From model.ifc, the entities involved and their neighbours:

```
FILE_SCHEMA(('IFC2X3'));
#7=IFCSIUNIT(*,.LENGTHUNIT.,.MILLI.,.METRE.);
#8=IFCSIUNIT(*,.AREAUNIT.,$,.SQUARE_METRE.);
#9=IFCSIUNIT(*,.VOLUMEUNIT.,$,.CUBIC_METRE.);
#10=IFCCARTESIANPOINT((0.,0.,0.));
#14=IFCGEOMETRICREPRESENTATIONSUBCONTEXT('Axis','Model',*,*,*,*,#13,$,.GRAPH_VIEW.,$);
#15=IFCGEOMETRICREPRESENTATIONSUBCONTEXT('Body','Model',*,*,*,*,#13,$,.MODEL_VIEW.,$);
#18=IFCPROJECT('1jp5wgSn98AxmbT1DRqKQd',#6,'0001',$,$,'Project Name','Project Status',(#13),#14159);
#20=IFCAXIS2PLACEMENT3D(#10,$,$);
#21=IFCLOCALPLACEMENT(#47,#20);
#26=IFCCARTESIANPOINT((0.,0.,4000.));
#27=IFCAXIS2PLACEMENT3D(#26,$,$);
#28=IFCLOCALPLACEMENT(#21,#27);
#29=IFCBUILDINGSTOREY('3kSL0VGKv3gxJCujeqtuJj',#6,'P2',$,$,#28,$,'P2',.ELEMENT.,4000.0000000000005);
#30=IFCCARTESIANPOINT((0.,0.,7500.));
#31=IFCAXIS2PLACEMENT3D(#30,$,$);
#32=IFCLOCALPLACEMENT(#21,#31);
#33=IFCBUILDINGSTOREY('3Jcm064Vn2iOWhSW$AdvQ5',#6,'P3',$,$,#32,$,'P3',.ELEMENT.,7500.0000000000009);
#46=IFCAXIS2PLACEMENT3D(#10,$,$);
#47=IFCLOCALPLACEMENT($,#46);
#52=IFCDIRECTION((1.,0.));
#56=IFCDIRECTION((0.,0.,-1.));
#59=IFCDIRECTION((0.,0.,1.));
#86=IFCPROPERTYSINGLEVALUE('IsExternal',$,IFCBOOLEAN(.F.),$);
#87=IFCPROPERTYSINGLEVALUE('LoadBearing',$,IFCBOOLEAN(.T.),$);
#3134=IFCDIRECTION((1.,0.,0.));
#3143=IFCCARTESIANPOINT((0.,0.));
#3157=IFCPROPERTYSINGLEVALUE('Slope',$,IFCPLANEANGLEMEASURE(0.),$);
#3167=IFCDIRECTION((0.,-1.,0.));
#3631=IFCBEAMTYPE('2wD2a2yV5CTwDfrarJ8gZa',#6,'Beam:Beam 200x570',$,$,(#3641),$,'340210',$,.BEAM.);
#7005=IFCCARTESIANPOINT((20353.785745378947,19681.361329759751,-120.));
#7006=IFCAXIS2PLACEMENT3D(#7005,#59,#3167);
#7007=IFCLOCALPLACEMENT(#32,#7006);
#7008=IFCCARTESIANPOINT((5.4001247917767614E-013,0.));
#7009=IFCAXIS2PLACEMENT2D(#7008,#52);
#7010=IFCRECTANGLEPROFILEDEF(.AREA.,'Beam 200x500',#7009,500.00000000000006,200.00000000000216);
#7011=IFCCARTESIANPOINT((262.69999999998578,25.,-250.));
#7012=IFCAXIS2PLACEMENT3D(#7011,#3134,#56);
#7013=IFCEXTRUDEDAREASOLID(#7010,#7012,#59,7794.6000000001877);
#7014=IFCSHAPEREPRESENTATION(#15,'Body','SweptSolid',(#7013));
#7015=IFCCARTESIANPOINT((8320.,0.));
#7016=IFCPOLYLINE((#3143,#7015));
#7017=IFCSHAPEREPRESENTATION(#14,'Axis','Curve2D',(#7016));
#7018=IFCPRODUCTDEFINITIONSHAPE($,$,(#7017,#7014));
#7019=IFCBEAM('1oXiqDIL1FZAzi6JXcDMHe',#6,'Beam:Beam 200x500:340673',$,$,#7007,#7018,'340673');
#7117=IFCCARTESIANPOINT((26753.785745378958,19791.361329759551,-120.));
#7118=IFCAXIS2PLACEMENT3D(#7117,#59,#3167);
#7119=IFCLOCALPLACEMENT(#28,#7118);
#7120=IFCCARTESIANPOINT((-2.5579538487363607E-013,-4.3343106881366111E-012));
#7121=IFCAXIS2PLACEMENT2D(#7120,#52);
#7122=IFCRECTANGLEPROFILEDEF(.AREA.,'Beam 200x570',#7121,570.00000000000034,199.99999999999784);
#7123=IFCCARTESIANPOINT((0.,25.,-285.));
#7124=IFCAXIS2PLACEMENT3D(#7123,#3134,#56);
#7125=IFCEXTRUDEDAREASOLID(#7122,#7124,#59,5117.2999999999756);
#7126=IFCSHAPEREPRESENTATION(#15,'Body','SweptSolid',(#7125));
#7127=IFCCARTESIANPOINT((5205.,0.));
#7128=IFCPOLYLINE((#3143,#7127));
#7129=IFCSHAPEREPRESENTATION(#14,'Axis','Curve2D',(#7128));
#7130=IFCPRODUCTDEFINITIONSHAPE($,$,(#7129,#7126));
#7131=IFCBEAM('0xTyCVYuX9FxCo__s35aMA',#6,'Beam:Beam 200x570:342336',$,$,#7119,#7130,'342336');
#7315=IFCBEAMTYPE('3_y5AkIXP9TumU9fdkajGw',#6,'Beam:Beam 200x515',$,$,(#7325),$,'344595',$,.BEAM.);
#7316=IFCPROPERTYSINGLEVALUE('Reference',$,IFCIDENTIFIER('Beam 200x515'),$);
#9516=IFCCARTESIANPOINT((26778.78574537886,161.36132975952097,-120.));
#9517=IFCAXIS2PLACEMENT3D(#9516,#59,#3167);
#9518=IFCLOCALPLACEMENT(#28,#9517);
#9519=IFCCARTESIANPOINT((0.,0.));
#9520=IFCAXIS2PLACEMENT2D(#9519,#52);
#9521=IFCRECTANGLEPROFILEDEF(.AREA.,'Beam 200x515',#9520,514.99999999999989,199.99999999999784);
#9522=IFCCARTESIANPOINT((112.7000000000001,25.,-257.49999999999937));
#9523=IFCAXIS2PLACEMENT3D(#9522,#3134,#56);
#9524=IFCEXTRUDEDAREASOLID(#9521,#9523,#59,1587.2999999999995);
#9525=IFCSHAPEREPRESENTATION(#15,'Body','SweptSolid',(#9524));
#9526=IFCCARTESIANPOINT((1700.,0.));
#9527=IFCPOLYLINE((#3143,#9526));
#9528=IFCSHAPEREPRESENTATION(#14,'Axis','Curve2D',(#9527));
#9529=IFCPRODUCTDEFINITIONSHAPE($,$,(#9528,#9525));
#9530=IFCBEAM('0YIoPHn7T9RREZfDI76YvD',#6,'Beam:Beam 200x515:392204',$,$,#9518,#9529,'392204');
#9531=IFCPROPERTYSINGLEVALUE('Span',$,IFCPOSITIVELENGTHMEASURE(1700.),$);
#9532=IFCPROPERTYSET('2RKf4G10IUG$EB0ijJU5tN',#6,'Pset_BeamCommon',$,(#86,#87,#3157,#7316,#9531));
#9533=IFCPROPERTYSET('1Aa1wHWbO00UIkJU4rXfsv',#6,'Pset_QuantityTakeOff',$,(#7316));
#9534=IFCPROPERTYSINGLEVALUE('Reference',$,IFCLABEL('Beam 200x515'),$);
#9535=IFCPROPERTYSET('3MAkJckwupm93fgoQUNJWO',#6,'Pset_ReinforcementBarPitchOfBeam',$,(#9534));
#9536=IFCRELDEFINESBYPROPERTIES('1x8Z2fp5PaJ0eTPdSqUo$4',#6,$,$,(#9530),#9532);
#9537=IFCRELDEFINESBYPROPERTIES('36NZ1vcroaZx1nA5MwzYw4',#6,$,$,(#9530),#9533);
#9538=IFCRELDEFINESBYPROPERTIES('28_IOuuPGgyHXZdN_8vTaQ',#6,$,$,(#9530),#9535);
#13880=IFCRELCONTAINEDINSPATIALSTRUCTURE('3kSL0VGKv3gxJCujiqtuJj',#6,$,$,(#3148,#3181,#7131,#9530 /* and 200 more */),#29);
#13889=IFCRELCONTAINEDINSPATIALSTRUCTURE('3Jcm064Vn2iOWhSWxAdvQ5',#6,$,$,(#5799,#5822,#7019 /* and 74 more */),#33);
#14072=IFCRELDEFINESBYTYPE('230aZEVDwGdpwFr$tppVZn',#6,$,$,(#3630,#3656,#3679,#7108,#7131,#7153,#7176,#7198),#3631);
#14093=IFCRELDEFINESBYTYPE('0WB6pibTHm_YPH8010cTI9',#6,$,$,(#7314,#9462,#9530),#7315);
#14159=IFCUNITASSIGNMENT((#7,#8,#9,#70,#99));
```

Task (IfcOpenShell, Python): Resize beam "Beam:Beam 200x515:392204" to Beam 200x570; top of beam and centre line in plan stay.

```python
import ifcopenshell
import ifcopenshell.api.pset
import ifcopenshell.api.type
import ifcopenshell.util.element
import ifcopenshell.util.representation

model = ifcopenshell.open("model.ifc")

member = model.by_guid("0YIoPHn7T9RREZfDI76YvD")
source = next(p for p in model.by_type("IfcRectangleProfileDef") if p.ProfileName == "Beam 200x570")

body = ifcopenshell.util.representation.get_representation(member, "Model", "Body")
solid = body.Items[0]
old_profile = solid.SweptArea

# Copy the section's sizes but keep this member's own profile position.
profile = ifcopenshell.util.element.copy(model, source)
# Profiles are centred, so shift by half the change in depth to hold the top.
shift = (old_profile.XDim - profile.XDim) / 2
x, y = old_profile.Position.Location.Coordinates
up = (-1.0, 0.0)  # upwards, in the solid's own plane
location = model.createIfcCartesianPoint((x + up[0] * shift, y + up[1] * shift))
profile.Position = model.createIfcAxis2Placement2D(location, old_profile.Position.RefDirection)
solid.SweptArea = profile
if not model.get_total_inverses(old_profile):
    ifcopenshell.util.element.remove_deep2(model, old_profile)

new_type = model.by_guid("2wD2a2yV5CTwDfrarJ8gZa")
ifcopenshell.api.type.assign_type(
    model, related_objects=[member], relating_type=new_type, should_map_representations=False
)
member.Name = member.Name.replace("Beam 200x515", "Beam 200x570")
pset = model.by_id(ifcopenshell.util.element.get_pset(member, "Pset_BeamCommon", should_inherit=False)["id"])
ifcopenshell.api.pset.edit_pset(model, pset=pset, properties={"Reference": "Beam 200x570"})
pset = model.by_id(ifcopenshell.util.element.get_pset(member, "Pset_QuantityTakeOff", should_inherit=False)["id"])
ifcopenshell.api.pset.edit_pset(model, pset=pset, properties={"Reference": "Beam 200x570"})
pset = model.by_id(ifcopenshell.util.element.get_pset(member, "Pset_ReinforcementBarPitchOfBeam", should_inherit=False)["id"])
ifcopenshell.api.pset.edit_pset(model, pset=pset, properties={"Reference": "Beam 200x570"})

print(solid.SweptArea)

model.write("model_v2.ifc")
```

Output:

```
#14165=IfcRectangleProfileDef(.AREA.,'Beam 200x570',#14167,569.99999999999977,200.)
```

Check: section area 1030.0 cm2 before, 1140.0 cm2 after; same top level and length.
